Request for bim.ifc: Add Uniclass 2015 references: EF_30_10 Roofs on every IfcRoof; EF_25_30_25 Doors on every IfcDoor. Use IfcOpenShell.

First a look at what the model holds.

```python
import ifcopenshell

model = ifcopenshell.open("bim.ifc")
print(model.schema)
print("classifications:", [c.Name for c in model.by_type("IfcClassification")])
for ifc_class in ("IfcDoor", "IfcRoof", "IfcStair", "IfcWall", "IfcWindow"):
    print(ifc_class, len(model.by_type(ifc_class)))
```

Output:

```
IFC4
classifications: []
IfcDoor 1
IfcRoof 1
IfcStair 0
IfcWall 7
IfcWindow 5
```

```python
import ifcopenshell
import ifcopenshell.api.classification

model = ifcopenshell.open("bim.ifc")

system = ifcopenshell.api.classification.add_classification(model, classification="Uniclass 2015")

codes = {
    "IfcRoof": ("EF_30_10", "Roofs"),
    "IfcDoor": ("EF_25_30_25", "Doors"),
}
for ifc_class, (code, name) in codes.items():
    products = model.by_type(ifc_class)
    ifcopenshell.api.classification.add_reference(
        model, products=products, classification=system, identification=code, name=name
    )
    print(code, len(products))

model.write("bim-out.ifc")
```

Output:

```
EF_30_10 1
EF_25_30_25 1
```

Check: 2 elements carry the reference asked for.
